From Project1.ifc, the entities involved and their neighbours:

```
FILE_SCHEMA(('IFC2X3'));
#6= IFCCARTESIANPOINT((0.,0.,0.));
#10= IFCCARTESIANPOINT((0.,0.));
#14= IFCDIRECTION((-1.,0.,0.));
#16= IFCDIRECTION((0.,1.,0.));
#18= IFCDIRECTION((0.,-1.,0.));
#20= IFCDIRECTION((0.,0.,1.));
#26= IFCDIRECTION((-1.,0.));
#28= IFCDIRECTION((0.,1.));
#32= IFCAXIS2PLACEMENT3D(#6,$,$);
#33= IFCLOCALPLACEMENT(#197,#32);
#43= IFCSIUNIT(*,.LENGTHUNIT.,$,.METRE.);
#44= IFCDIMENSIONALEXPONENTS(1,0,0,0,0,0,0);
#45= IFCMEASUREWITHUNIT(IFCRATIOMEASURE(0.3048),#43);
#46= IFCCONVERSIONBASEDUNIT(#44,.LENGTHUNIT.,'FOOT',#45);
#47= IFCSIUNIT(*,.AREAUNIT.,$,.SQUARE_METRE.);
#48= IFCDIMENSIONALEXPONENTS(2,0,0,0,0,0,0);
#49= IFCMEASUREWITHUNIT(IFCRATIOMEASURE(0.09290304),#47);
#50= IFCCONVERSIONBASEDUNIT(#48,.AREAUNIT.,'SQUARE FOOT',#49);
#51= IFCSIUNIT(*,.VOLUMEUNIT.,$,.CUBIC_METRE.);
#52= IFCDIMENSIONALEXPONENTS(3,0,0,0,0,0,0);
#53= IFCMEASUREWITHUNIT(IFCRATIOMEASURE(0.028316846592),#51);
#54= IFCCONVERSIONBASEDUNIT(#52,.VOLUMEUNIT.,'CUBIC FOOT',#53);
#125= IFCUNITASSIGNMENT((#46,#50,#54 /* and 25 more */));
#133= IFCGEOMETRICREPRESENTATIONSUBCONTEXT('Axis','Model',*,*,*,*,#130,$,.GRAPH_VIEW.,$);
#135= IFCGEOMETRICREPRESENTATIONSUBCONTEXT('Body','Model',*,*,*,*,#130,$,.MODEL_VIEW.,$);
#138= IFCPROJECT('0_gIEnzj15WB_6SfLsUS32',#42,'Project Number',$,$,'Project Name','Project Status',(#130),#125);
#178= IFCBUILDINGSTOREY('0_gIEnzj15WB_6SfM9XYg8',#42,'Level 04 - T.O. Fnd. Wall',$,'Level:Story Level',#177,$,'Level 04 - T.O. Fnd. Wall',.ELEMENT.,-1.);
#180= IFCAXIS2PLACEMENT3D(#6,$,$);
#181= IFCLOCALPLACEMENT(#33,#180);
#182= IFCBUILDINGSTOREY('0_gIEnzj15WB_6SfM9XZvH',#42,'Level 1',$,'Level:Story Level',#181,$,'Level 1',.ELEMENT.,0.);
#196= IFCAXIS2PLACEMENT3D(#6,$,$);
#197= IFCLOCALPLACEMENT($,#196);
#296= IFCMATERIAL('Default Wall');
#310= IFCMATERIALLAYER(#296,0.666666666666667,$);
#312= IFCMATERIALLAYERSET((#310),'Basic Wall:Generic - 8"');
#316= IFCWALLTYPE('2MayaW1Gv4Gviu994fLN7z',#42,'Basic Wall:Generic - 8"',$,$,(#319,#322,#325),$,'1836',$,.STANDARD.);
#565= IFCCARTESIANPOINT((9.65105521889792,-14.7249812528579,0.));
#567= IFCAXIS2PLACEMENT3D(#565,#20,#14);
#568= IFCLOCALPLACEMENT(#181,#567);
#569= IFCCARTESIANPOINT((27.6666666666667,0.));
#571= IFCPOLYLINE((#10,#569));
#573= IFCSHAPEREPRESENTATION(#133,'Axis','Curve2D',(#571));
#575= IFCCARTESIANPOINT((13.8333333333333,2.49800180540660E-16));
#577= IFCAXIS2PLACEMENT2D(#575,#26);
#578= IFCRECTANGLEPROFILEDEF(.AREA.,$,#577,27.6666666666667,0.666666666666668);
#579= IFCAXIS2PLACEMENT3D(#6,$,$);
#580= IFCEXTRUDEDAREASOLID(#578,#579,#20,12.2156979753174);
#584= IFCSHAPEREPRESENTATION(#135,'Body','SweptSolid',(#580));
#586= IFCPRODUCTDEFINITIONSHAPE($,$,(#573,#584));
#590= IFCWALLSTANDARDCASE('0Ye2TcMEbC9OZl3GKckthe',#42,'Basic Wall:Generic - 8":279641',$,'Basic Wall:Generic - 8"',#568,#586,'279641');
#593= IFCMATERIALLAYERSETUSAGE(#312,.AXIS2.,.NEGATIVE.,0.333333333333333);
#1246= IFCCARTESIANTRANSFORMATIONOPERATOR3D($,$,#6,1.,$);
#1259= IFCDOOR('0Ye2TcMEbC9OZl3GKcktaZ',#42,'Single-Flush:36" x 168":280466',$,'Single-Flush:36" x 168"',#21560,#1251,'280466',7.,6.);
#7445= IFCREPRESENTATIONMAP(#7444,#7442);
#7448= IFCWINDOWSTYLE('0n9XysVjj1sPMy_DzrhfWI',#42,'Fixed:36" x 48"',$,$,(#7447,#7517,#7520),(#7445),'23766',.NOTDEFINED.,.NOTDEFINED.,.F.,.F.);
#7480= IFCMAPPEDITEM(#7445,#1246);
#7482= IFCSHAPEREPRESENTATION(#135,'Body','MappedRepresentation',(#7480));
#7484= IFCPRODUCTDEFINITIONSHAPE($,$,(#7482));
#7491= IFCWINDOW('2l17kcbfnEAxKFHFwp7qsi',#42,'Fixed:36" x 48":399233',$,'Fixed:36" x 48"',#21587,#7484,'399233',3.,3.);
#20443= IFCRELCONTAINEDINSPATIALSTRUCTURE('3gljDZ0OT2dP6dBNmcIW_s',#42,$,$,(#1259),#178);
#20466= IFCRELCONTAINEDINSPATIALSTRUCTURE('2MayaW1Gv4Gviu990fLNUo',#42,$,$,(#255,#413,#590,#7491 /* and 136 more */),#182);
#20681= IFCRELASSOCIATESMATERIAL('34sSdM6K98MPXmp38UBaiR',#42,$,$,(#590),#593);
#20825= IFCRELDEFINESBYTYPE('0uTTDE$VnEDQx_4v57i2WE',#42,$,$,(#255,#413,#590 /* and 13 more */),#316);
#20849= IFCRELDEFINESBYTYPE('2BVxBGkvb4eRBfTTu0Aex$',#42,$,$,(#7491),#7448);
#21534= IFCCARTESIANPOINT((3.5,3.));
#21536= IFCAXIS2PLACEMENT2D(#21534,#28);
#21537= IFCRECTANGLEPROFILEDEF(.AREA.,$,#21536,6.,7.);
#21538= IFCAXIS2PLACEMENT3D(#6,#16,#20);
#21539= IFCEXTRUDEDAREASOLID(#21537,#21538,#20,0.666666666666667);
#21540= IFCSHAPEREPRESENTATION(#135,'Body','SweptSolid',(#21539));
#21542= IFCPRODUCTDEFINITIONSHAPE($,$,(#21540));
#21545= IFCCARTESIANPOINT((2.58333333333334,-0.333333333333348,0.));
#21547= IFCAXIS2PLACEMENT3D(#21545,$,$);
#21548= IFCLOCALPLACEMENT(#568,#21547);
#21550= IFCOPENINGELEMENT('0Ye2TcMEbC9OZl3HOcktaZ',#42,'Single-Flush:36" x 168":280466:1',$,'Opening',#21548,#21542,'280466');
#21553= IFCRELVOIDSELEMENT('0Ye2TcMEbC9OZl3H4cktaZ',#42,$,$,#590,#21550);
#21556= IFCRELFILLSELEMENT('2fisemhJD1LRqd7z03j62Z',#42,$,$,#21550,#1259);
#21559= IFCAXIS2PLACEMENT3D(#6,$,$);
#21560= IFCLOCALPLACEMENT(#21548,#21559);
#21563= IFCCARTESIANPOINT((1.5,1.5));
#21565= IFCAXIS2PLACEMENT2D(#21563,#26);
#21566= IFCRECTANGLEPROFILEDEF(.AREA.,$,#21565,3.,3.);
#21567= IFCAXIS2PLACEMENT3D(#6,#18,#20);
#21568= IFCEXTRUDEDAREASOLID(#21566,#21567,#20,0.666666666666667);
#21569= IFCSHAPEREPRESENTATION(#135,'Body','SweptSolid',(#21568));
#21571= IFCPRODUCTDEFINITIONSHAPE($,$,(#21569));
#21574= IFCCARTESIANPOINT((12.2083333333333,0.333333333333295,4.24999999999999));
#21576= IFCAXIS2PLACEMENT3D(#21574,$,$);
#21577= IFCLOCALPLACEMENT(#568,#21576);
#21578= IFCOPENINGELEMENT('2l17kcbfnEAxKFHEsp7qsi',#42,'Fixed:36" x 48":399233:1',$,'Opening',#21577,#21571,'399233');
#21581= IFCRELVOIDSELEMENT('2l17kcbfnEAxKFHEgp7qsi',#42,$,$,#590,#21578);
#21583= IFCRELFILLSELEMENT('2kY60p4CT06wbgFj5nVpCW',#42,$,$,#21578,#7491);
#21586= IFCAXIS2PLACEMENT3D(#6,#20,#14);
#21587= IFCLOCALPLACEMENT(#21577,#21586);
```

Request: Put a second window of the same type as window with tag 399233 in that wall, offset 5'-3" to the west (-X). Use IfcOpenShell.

```python
import ifcopenshell
import ifcopenshell.api.feature
import ifcopenshell.api.geometry
import ifcopenshell.api.root
import ifcopenshell.geom
import ifcopenshell.util.element
import ifcopenshell.util.placement
import ifcopenshell.util.shape
import ifcopenshell.util.unit

model = ifcopenshell.open("Project1.ifc")
unit_scale = ifcopenshell.util.unit.calculate_unit_scale(model)
settings = ifcopenshell.geom.settings()


def volume(element):
    """Net volume in cubic metres, openings subtracted."""
    shape = ifcopenshell.geom.create_shape(settings, element)
    return ifcopenshell.util.shape.get_volume(shape.geometry)


def reuse_history(source, copy):
    """copy_class also copies each property set's owner history, people and application; keep the originals."""
    for rel in copy.IsDefinedBy:
        if rel.is_a("IfcRelDefinesByProperties") and (history := rel.RelatingPropertyDefinition.OwnerHistory):
            rel.RelatingPropertyDefinition.OwnerHistory = source.OwnerHistory
            ifcopenshell.util.element.remove_deep2(model, history)


window = model.by_guid("2l17kcbfnEAxKFHFwp7qsi")
opening = window.FillsVoids[0].RelatingOpeningElement
wall = opening.VoidsElements[0].RelatingBuildingElement
before = volume(wall)
shift = ifcopenshell.util.placement.get_local_placement(wall.ObjectPlacement)[:3, 0] * 63 * 0.0254 / unit_scale

# copy_class copies the void relationship, type, container and properties, but no geometry.
new_opening = ifcopenshell.api.root.copy_class(model, product=opening)
new_opening.Representation = ifcopenshell.util.element.copy_deep(
    model, opening.Representation, exclude=["IfcGeometricRepresentationContext", "IfcRepresentationMap"]
)
new_opening.Name = 'Fixed:36" x 48"'
new_opening.Tag = None
new_window = ifcopenshell.api.root.copy_class(model, product=window)
new_window.Representation = ifcopenshell.util.element.copy_deep(
    model, window.Representation, exclude=["IfcGeometricRepresentationContext", "IfcRepresentationMap"]
)
new_window.Name = 'Fixed:36" x 48"'
new_window.Tag = None
reuse_history(window, new_window)
fills = ifcopenshell.api.feature.add_filling(model, opening=new_opening, element=new_window)
fills.OwnerHistory = new_window.OwnerHistory  # required in IFC2X3

for old, new in ((opening, new_opening), (window, new_window)):
    matrix = ifcopenshell.util.placement.get_local_placement(old.ObjectPlacement)
    matrix[:3, 3] += shift
    ifcopenshell.api.geometry.edit_object_placement(model, product=new, matrix=matrix, is_si=False)

after = volume(wall)

print(f"wall volume {before:.3f} -> {after:.3f} m3")

model.write("Project1_edited.ifc")
```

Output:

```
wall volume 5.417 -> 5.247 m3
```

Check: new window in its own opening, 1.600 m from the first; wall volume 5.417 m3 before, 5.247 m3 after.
